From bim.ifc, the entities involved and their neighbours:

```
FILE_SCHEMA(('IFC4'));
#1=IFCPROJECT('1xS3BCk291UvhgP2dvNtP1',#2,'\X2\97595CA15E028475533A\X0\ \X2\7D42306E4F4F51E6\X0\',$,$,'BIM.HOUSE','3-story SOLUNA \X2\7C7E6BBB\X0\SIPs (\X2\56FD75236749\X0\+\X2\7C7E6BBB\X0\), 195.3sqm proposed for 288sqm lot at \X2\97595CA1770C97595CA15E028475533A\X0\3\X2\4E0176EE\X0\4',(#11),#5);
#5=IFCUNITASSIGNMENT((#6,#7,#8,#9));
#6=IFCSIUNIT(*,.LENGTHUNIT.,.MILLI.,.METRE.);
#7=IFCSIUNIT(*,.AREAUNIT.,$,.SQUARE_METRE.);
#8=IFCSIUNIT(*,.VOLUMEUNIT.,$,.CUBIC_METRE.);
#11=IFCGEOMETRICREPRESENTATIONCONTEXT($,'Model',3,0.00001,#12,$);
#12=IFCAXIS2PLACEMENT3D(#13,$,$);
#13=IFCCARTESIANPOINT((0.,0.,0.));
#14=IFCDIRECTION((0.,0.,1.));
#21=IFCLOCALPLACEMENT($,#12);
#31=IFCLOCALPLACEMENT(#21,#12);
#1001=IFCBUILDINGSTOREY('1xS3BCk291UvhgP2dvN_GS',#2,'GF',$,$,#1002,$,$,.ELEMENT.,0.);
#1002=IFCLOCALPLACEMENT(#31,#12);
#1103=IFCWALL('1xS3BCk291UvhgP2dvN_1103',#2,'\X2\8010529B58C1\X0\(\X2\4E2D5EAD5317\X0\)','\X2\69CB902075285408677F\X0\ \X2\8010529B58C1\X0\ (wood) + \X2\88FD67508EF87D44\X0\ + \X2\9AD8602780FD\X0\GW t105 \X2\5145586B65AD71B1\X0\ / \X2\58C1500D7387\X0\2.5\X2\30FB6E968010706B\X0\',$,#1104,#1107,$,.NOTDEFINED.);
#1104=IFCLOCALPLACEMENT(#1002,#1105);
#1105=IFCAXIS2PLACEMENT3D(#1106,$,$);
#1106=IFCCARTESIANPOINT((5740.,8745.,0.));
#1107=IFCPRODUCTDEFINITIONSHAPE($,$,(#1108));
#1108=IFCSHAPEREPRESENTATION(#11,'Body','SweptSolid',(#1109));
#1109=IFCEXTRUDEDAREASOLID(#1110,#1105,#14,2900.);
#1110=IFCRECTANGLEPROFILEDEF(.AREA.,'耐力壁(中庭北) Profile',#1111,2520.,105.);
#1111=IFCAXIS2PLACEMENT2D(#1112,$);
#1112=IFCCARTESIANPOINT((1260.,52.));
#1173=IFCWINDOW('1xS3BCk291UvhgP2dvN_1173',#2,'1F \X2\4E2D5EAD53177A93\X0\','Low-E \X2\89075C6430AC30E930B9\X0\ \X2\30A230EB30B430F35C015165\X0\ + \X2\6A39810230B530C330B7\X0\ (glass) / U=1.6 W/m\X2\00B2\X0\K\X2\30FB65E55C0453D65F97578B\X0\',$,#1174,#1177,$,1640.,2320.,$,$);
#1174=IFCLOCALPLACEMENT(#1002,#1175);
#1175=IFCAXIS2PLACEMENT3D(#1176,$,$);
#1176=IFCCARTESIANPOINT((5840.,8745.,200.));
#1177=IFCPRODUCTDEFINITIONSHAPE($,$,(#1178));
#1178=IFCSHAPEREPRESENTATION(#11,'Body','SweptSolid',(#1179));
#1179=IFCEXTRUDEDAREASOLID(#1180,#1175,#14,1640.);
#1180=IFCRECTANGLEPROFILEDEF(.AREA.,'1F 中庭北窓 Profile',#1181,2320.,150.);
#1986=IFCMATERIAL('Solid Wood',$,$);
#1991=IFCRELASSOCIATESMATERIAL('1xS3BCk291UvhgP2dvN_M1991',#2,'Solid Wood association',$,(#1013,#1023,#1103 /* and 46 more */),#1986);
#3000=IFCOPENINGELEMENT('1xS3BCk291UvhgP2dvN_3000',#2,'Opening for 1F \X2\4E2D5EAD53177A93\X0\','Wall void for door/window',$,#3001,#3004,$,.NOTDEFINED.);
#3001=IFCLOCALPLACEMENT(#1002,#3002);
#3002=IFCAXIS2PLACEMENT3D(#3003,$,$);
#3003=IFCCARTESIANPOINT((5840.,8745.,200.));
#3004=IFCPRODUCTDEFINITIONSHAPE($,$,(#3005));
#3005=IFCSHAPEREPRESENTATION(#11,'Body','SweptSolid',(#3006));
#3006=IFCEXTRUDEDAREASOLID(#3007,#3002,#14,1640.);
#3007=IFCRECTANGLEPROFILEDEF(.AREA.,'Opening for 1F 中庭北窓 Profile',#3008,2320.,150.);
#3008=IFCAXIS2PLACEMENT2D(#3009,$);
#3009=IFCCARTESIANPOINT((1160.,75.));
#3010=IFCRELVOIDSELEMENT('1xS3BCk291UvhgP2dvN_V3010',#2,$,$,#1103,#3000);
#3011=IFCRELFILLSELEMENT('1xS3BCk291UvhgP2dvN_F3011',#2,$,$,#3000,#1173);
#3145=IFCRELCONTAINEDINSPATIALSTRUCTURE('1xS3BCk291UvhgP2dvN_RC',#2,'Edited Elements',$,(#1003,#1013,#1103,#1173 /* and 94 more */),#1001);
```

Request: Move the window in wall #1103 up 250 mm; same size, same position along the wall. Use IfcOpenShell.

```python
import numpy as np
import ifcopenshell
import ifcopenshell.api.geometry
import ifcopenshell.util.placement
import ifcopenshell.util.unit

model = ifcopenshell.open("bim.ifc")
unit_scale = ifcopenshell.util.unit.calculate_unit_scale(model)

window = model.by_guid("1xS3BCk291UvhgP2dvN_1173")
opening = window.FillsVoids[0].RelatingOpeningElement
dz = 250.0

shift = np.array([0.0, 0.0, dz])
# The window is not placed relative to its opening, so move both.
for product in (opening, window):
    matrix = ifcopenshell.util.placement.get_local_placement(product.ObjectPlacement)
    matrix[:3, 3] += shift
    ifcopenshell.api.geometry.edit_object_placement(model, product=product, matrix=matrix, is_si=False)

print(f"moved by {dz * unit_scale:+.3f} m")

model.write("bim_edited.ifc")
```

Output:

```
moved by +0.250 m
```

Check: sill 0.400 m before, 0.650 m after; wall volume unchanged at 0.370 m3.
